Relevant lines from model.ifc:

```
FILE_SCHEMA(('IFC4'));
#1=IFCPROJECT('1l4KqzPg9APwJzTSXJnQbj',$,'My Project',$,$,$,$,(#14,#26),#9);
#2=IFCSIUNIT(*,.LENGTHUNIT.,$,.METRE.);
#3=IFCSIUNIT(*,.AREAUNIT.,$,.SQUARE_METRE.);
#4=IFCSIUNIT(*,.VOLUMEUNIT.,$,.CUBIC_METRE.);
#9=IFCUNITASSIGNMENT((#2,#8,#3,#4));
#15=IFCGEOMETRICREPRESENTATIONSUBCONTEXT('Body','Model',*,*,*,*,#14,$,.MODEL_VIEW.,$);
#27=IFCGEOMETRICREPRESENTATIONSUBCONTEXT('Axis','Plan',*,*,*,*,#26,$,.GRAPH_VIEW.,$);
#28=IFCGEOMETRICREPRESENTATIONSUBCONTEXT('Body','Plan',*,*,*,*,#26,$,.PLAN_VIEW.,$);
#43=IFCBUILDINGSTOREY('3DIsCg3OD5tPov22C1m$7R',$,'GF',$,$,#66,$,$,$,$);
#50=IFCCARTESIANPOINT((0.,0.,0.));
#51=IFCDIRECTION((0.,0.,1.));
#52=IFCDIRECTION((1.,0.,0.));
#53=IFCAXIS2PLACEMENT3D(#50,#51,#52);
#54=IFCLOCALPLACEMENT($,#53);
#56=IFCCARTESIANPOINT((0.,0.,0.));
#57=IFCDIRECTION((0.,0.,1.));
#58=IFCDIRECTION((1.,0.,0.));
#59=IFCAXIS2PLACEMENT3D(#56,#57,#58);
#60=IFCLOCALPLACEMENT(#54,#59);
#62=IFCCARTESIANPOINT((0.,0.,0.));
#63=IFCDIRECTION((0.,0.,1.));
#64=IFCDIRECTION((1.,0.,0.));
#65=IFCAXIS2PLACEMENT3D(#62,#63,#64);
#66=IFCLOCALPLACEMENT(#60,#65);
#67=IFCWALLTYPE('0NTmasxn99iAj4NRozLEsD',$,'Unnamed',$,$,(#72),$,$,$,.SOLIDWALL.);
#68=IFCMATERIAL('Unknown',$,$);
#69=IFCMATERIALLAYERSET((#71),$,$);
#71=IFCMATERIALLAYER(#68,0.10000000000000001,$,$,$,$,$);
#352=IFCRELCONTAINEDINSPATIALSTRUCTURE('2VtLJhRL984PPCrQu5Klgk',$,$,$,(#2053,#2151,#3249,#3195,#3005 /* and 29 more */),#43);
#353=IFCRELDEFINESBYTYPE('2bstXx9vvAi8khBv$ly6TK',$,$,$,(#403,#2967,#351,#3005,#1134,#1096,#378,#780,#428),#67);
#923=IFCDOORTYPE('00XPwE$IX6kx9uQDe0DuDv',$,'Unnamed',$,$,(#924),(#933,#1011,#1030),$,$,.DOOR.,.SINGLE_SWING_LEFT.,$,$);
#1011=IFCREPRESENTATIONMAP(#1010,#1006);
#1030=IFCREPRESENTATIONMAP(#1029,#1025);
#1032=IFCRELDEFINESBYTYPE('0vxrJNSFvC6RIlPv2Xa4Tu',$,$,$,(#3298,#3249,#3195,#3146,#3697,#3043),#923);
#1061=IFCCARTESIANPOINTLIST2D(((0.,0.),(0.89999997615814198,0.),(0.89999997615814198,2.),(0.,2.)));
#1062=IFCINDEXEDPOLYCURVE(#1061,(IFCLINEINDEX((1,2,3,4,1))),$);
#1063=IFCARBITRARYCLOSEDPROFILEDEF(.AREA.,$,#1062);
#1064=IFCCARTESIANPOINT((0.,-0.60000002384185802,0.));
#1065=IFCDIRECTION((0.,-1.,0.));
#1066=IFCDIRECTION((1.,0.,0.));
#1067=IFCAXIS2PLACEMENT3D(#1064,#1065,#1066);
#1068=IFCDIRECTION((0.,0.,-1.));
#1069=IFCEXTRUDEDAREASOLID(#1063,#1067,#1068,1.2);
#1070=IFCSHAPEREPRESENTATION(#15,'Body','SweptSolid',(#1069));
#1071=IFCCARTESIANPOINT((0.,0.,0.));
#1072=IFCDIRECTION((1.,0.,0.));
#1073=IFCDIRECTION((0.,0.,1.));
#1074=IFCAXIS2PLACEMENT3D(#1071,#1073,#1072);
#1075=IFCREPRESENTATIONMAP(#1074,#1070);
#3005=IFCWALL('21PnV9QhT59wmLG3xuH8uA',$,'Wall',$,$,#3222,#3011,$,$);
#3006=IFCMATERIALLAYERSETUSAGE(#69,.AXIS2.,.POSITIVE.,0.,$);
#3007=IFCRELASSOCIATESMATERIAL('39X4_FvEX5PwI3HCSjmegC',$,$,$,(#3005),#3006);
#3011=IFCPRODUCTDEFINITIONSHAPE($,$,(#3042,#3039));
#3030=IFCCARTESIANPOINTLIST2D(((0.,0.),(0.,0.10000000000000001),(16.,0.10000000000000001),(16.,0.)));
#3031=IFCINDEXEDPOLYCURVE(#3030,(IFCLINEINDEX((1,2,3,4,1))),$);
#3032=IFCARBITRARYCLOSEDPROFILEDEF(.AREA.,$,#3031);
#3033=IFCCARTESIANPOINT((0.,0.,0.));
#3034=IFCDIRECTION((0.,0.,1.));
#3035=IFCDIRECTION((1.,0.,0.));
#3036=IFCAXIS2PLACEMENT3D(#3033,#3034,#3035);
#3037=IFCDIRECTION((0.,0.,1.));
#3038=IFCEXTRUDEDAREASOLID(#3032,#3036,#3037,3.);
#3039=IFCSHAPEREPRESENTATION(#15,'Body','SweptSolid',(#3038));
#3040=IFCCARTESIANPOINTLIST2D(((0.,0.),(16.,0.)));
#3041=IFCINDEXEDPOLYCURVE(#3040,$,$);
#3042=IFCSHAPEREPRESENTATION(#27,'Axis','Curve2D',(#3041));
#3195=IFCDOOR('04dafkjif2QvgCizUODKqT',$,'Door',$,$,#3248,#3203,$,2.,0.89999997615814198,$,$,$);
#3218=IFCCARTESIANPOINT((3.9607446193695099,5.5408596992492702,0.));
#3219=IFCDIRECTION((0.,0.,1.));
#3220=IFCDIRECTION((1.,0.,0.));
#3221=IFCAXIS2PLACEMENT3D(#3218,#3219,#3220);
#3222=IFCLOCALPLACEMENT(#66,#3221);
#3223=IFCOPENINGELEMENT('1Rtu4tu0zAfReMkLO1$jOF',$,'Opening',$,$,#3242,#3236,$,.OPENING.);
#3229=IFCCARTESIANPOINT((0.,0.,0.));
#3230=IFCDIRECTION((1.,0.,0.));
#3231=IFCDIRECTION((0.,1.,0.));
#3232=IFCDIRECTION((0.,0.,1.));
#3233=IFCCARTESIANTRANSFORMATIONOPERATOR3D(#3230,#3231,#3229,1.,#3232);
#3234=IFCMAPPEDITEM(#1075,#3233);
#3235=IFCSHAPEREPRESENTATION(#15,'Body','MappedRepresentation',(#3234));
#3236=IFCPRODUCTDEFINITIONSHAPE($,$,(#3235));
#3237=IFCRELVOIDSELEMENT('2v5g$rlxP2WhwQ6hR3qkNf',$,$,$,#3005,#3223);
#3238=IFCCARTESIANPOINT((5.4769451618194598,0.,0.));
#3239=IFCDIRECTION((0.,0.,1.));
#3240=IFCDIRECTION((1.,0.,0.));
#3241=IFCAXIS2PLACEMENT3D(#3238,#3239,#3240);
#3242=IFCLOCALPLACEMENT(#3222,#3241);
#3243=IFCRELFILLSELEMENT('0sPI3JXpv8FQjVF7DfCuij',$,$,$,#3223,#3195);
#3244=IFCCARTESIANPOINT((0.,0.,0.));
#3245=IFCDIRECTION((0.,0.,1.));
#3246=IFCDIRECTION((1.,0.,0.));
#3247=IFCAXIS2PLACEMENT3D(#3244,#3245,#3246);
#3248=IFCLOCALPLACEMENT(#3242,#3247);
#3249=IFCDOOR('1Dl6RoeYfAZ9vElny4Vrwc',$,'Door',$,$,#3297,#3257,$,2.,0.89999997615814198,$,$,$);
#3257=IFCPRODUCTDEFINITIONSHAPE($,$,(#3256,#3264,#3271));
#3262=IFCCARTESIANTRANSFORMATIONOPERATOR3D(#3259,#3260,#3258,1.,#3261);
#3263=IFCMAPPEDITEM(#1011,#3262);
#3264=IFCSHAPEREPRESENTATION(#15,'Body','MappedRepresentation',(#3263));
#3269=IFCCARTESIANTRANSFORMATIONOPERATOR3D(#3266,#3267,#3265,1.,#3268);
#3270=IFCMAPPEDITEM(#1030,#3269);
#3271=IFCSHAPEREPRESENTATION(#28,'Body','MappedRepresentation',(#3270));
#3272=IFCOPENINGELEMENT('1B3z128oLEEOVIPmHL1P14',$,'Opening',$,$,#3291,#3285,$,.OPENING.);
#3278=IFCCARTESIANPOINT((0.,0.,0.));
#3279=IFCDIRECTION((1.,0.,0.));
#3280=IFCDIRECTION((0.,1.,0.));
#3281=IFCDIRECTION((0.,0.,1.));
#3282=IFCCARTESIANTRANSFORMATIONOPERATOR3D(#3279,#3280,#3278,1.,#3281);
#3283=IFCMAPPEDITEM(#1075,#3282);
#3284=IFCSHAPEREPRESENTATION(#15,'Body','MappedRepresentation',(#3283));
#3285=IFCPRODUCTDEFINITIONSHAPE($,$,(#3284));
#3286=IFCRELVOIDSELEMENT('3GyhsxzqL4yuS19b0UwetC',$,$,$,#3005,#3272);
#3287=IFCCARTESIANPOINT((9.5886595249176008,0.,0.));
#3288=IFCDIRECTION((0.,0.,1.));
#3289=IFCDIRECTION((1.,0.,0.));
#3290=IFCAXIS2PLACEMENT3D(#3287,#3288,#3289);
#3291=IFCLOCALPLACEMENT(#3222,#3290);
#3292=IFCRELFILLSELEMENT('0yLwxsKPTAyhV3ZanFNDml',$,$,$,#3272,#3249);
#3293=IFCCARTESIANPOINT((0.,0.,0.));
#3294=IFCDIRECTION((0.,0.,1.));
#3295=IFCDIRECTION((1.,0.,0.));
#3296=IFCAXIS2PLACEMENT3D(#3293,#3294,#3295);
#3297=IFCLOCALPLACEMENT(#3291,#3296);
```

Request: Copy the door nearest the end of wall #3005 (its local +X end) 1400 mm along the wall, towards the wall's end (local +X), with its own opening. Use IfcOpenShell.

```python
import ifcopenshell
import ifcopenshell.api.feature
import ifcopenshell.api.geometry
import ifcopenshell.api.root
import ifcopenshell.geom
import ifcopenshell.util.element
import ifcopenshell.util.placement
import ifcopenshell.util.shape

model = ifcopenshell.open("model.ifc")
settings = ifcopenshell.geom.settings()


def volume(element):
    """Net volume in cubic metres, openings subtracted."""
    shape = ifcopenshell.geom.create_shape(settings, element)
    return ifcopenshell.util.shape.get_volume(shape.geometry)


door = model.by_guid("1Dl6RoeYfAZ9vElny4Vrwc")
opening = door.FillsVoids[0].RelatingOpeningElement
wall = opening.VoidsElements[0].RelatingBuildingElement
before = volume(wall)
shift = ifcopenshell.util.placement.get_local_placement(wall.ObjectPlacement)[:3, 0] * 1.4

# copy_class copies the void relationship, type, container and properties, but no geometry.
new_opening = ifcopenshell.api.root.copy_class(model, product=opening)
new_opening.Representation = ifcopenshell.util.element.copy_deep(
    model, opening.Representation, exclude=["IfcGeometricRepresentationContext", "IfcRepresentationMap"]
)
new_door = ifcopenshell.api.root.copy_class(model, product=door)
new_door.Representation = ifcopenshell.util.element.copy_deep(
    model, door.Representation, exclude=["IfcGeometricRepresentationContext", "IfcRepresentationMap"]
)
ifcopenshell.api.feature.add_filling(model, opening=new_opening, element=new_door)

for old, new in ((opening, new_opening), (door, new_door)):
    matrix = ifcopenshell.util.placement.get_local_placement(old.ObjectPlacement)
    matrix[:3, 3] += shift
    ifcopenshell.api.geometry.edit_object_placement(model, product=new, matrix=matrix, is_si=False)

after = volume(wall)

print(f"wall volume {before:.3f} -> {after:.3f} m3")

model.write("model_v2.ifc")
```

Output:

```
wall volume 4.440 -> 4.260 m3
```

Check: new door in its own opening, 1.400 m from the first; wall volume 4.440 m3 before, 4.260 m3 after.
